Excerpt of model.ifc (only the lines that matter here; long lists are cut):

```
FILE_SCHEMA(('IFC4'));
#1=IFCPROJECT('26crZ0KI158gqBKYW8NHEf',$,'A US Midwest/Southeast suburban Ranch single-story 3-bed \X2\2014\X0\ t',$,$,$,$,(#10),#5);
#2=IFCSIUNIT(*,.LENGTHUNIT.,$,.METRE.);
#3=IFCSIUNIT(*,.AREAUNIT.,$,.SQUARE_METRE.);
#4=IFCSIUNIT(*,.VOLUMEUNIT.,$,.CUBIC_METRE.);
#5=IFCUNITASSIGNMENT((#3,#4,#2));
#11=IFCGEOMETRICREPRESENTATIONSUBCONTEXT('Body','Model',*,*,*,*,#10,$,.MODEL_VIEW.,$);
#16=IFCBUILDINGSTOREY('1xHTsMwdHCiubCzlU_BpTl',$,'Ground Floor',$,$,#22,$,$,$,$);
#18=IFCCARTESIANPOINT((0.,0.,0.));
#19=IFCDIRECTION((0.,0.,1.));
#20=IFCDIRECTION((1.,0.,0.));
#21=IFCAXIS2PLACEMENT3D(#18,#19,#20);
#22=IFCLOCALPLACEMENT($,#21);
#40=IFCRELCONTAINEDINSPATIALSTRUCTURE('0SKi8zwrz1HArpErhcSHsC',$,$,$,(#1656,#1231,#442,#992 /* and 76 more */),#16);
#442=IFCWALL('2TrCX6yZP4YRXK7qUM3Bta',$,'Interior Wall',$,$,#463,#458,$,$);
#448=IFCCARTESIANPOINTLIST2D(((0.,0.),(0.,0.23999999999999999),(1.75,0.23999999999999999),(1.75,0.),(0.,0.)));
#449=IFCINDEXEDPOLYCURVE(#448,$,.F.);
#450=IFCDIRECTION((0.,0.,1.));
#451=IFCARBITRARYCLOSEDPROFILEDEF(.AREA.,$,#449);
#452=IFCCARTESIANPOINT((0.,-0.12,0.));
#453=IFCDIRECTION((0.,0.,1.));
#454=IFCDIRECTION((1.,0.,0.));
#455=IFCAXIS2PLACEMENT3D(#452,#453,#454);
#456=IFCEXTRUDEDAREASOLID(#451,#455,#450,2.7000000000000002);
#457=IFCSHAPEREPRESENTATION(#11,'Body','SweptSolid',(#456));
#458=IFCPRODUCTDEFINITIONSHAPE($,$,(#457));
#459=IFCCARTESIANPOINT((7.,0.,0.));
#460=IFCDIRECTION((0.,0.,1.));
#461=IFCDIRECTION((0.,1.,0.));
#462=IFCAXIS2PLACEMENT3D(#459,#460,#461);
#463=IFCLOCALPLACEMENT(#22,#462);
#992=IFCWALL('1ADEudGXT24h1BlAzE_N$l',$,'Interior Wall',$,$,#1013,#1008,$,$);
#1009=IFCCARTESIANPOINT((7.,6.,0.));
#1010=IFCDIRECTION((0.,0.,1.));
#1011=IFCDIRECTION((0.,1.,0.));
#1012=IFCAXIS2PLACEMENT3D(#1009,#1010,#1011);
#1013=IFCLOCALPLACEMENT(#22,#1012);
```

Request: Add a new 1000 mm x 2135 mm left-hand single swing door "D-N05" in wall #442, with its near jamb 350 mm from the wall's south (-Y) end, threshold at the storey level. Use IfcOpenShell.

```python
import numpy as np
import ifcopenshell
import ifcopenshell.api.feature
import ifcopenshell.api.geometry
import ifcopenshell.api.root
import ifcopenshell.api.spatial
import ifcopenshell.geom
import ifcopenshell.util.element
import ifcopenshell.util.placement
import ifcopenshell.util.representation
import ifcopenshell.util.shape
import ifcopenshell.util.unit

model = ifcopenshell.open("model.ifc")
unit_scale = ifcopenshell.util.unit.calculate_unit_scale(model)
settings = ifcopenshell.geom.settings()


def volume(element):
    """Net volume in cubic metres, openings subtracted."""
    shape = ifcopenshell.geom.create_shape(settings, element)
    return ifcopenshell.util.shape.get_volume(shape.geometry)


wall = model.by_guid("2TrCX6yZP4YRXK7qUM3Bta")
storey = ifcopenshell.util.element.get_container(wall, ifc_class="IfcBuildingStorey")
context = ifcopenshell.util.representation.get_context(model, "Model", "Body", "MODEL_VIEW")
before = volume(wall)

width, height, from_end, sill = 1, 2.135, 0.35, 0.0  # metres

# The wall runs along its own X axis, and the end named is its -X end.
wall_shape = ifcopenshell.geom.create_shape(settings, wall)
x, y, z = ifcopenshell.util.shape.get_vertices(wall_shape.geometry).T
start = x.min() + from_end
face, thickness = float(y.min()), float(y.max() - y.min())
wall_matrix = ifcopenshell.util.placement.get_local_placement(wall.ObjectPlacement)
level = ifcopenshell.util.placement.get_local_placement(storey.ObjectPlacement)[2, 3]


def in_wall(x, y):
    """Placement at x, y metres in the wall's axes, at sill height."""
    matrix = wall_matrix.copy()
    matrix[:, 3] = wall_matrix @ np.array([x / unit_scale, y / unit_scale, 0.0, 1.0])
    matrix[2, 3] = level + sill / unit_scale
    return matrix


# Opening: a box that overshoots both wall faces by 50 mm.
opening = ifcopenshell.api.root.create_entity(model, ifc_class="IfcOpeningElement", predefined_type="OPENING")
box = ifcopenshell.api.geometry.add_wall_representation(
    model, context=context, length=width, height=height, thickness=thickness + 0.1
)
ifcopenshell.api.geometry.assign_representation(model, product=opening, representation=box)
ifcopenshell.api.geometry.edit_object_placement(model, product=opening, matrix=in_wall(start, face - 0.05), is_si=False)
ifcopenshell.api.feature.add_feature(model, feature=opening, element=wall)

door = ifcopenshell.api.root.create_entity(model, ifc_class="IfcDoor", name="D-N05", predefined_type="DOOR")
door.OverallWidth, door.OverallHeight = width / unit_scale, height / unit_scale
door.OperationType = "SINGLE_SWING_LEFT"
body = ifcopenshell.api.geometry.add_door_representation(
    model,
    context=context,
    overall_width=door.OverallWidth,
    overall_height=door.OverallHeight,
    operation_type="SINGLE_SWING_LEFT",
    lining_properties={"LiningDepth": thickness / unit_scale, "ThresholdDepth": thickness / unit_scale},
)
ifcopenshell.api.geometry.assign_representation(model, product=door, representation=body)
ifcopenshell.api.spatial.assign_container(model, products=[door], relating_structure=storey)
ifcopenshell.api.feature.add_filling(model, opening=opening, element=door)

# The lining spans the wall, so the door starts at the wall face.
ifcopenshell.api.geometry.edit_object_placement(model, product=door, matrix=in_wall(start, face), is_si=False)

after = volume(wall)

print(f"wall volume {before:.3f} -> {after:.3f} m3")

model.write("model_rev.ifc")
```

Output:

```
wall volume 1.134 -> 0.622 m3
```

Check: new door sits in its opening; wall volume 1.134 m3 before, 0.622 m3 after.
